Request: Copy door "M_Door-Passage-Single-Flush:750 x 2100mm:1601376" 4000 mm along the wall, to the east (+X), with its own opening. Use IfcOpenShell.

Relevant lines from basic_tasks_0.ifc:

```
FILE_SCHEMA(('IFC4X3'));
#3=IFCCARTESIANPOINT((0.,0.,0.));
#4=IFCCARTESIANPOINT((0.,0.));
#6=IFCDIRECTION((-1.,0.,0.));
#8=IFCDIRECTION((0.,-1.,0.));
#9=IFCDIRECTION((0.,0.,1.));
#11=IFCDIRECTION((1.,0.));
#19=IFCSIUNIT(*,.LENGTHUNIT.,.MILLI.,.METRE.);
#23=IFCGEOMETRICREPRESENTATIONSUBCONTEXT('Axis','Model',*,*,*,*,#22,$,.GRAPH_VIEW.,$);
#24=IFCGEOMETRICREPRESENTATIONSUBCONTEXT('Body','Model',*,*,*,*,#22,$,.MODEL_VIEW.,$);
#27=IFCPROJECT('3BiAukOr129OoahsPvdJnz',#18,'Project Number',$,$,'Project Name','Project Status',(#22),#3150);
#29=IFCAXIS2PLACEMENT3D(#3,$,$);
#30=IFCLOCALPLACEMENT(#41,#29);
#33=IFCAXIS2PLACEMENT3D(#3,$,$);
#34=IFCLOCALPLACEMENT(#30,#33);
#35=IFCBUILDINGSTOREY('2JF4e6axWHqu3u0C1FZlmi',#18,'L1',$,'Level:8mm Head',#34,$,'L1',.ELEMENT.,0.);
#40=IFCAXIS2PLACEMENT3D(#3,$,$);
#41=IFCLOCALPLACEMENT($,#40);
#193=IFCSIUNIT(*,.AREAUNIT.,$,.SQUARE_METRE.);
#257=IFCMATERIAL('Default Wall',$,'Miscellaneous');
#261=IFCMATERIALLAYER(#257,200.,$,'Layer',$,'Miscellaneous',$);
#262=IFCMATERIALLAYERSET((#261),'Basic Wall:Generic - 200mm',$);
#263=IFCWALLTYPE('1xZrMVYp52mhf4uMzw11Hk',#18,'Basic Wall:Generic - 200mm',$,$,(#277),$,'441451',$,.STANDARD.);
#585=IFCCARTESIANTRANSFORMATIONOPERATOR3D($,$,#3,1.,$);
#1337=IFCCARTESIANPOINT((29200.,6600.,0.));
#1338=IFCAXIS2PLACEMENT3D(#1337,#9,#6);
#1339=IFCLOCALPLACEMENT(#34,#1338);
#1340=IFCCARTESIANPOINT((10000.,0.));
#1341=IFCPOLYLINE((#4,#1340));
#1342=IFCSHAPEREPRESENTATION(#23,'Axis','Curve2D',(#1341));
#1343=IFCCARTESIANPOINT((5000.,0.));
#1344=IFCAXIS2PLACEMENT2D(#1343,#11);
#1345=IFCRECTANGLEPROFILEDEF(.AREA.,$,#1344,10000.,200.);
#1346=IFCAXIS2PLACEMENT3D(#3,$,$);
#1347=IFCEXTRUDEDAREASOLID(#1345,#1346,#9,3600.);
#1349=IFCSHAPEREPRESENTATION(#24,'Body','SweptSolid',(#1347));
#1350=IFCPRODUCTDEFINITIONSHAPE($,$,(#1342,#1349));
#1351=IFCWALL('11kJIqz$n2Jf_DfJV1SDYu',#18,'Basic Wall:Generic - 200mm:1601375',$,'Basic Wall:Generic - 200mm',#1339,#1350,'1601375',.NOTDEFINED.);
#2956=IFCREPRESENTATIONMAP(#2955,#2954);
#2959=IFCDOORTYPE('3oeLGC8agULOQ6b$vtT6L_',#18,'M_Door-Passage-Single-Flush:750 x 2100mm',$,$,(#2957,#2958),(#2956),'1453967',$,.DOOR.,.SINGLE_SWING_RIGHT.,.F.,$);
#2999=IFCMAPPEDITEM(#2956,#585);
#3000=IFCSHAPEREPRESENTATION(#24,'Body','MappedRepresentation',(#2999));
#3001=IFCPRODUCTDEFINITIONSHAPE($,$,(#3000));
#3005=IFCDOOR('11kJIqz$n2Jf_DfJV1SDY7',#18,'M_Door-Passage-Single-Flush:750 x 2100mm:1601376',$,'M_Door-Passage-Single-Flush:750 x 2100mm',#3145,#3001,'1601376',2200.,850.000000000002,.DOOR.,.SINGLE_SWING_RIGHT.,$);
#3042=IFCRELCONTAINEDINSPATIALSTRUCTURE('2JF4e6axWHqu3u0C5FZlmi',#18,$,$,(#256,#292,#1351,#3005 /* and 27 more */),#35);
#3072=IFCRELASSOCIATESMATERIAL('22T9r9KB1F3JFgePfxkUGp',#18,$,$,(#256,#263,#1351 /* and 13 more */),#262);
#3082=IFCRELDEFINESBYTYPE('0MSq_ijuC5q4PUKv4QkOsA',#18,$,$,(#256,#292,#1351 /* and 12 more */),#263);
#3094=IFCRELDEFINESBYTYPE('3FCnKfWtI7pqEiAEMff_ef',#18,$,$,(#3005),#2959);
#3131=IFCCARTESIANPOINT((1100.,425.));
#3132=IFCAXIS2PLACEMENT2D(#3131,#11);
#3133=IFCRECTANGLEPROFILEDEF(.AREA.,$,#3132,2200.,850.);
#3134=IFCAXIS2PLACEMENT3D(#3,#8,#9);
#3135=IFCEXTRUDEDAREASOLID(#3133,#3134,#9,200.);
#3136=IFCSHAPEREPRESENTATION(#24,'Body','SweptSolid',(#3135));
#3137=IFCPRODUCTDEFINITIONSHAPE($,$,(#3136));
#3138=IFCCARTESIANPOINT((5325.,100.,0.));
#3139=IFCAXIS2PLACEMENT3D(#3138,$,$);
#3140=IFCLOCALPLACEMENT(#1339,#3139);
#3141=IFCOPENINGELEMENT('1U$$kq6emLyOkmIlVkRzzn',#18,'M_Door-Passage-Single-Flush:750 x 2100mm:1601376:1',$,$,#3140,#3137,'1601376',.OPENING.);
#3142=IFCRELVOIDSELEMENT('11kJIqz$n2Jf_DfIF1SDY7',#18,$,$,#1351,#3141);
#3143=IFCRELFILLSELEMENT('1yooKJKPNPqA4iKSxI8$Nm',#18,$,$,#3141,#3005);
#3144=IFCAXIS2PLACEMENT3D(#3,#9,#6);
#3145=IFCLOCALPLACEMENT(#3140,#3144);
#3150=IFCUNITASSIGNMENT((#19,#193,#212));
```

```python
import ifcopenshell
import ifcopenshell.api.feature
import ifcopenshell.api.geometry
import ifcopenshell.api.root
import ifcopenshell.geom
import ifcopenshell.util.element
import ifcopenshell.util.placement
import ifcopenshell.util.shape
import ifcopenshell.util.unit

model = ifcopenshell.open("basic_tasks_0.ifc")
unit_scale = ifcopenshell.util.unit.calculate_unit_scale(model)
settings = ifcopenshell.geom.settings()


def volume(element):
    """Net volume in cubic metres, openings subtracted."""
    shape = ifcopenshell.geom.create_shape(settings, element)
    return ifcopenshell.util.shape.get_volume(shape.geometry)


def reuse_history(source, copy):
    """copy_class also copies each property set's owner history, people and application; keep the originals."""
    for rel in copy.IsDefinedBy:
        if rel.is_a("IfcRelDefinesByProperties") and (history := rel.RelatingPropertyDefinition.OwnerHistory):
            rel.RelatingPropertyDefinition.OwnerHistory = source.OwnerHistory
            ifcopenshell.util.element.remove_deep2(model, history)


door = model.by_guid("11kJIqz$n2Jf_DfJV1SDY7")
opening = door.FillsVoids[0].RelatingOpeningElement
wall = opening.VoidsElements[0].RelatingBuildingElement
before = volume(wall)
shift = ifcopenshell.util.placement.get_local_placement(wall.ObjectPlacement)[:3, 0] * -4 / unit_scale

# copy_class copies the void relationship, type, container and properties, but no geometry.
new_opening = ifcopenshell.api.root.copy_class(model, product=opening)
new_opening.Representation = ifcopenshell.util.element.copy_deep(
    model, opening.Representation, exclude=["IfcGeometricRepresentationContext", "IfcRepresentationMap"]
)
new_opening.Name = "M_Door-Passage-Single-Flush:750 x 2100mm"
new_opening.Tag = None
new_door = ifcopenshell.api.root.copy_class(model, product=door)
new_door.Representation = ifcopenshell.util.element.copy_deep(
    model, door.Representation, exclude=["IfcGeometricRepresentationContext", "IfcRepresentationMap"]
)
new_door.Name = "M_Door-Passage-Single-Flush:750 x 2100mm"
new_door.Tag = None
reuse_history(door, new_door)
ifcopenshell.api.feature.add_filling(model, opening=new_opening, element=new_door)

for old, new in ((opening, new_opening), (door, new_door)):
    matrix = ifcopenshell.util.placement.get_local_placement(old.ObjectPlacement)
    matrix[:3, 3] += shift
    ifcopenshell.api.geometry.edit_object_placement(model, product=new, matrix=matrix, is_si=False)

after = volume(wall)

print(f"wall volume {before:.3f} -> {after:.3f} m3")

model.write("basic_tasks_0_rev.ifc")
```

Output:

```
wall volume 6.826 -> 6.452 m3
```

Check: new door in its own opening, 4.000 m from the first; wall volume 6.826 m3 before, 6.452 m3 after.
